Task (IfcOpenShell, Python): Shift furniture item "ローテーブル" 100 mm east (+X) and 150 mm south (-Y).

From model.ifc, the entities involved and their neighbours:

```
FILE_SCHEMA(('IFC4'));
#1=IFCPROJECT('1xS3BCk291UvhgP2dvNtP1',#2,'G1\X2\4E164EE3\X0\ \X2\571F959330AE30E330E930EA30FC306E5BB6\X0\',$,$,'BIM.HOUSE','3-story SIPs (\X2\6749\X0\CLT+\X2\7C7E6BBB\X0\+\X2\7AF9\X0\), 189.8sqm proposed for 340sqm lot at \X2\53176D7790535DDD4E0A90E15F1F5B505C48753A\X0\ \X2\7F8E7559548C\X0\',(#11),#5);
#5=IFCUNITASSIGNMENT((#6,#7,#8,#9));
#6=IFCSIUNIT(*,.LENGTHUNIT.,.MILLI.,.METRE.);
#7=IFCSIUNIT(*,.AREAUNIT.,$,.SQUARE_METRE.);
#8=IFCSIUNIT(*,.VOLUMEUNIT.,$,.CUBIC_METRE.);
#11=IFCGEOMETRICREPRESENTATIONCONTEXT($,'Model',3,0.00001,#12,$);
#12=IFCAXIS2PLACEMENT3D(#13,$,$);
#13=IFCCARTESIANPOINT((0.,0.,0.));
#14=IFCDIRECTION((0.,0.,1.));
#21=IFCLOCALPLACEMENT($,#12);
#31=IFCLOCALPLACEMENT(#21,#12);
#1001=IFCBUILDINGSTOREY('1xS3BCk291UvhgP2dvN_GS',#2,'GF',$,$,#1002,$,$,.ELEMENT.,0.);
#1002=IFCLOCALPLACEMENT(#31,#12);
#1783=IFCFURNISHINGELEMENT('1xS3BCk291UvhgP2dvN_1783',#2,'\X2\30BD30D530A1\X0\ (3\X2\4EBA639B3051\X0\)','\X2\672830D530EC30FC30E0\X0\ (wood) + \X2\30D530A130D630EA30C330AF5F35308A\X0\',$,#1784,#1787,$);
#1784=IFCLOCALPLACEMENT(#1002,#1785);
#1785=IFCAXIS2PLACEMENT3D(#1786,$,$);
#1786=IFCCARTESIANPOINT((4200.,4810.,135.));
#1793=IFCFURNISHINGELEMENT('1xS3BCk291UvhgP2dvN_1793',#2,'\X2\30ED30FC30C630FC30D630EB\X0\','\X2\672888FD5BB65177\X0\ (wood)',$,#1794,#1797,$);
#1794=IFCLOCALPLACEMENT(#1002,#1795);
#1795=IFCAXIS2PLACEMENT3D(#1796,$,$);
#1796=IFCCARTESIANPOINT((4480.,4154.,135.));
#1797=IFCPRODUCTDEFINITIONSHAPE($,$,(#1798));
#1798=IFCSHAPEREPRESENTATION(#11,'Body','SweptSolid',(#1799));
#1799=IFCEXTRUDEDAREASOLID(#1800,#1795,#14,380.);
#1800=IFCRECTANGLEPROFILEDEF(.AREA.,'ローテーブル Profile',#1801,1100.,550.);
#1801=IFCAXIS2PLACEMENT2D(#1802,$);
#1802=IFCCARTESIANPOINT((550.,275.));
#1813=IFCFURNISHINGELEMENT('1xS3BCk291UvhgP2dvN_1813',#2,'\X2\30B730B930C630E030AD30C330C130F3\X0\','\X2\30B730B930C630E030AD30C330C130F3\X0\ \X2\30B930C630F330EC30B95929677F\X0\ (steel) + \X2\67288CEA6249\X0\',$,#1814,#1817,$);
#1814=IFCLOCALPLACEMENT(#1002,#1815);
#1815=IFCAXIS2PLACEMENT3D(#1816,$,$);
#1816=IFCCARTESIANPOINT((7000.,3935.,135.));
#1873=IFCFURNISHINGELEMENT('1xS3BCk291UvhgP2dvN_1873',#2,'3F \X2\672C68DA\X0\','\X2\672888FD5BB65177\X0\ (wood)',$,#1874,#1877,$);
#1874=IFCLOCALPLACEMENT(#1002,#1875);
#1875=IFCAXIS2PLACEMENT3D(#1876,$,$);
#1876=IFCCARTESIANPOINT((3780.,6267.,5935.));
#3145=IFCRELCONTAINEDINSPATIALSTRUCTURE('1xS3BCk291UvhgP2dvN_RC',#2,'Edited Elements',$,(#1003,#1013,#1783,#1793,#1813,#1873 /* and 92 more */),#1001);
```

```python
import ifcopenshell
import ifcopenshell.api.geometry
import ifcopenshell.util.placement
import ifcopenshell.util.unit

model = ifcopenshell.open("model.ifc")
unit_scale = ifcopenshell.util.unit.calculate_unit_scale(model)

item = model.by_guid("1xS3BCk291UvhgP2dvN_1793")
matrix = ifcopenshell.util.placement.get_local_placement(item.ObjectPlacement)
matrix[0, 3] += 0.1 / unit_scale
matrix[1, 3] -= 0.15 / unit_scale
ifcopenshell.api.geometry.edit_object_placement(model, product=item, matrix=matrix, is_si=False)

print(ifcopenshell.util.placement.get_local_placement(item.ObjectPlacement).round(3) + 0.0)

model.write("model-out.ifc")
```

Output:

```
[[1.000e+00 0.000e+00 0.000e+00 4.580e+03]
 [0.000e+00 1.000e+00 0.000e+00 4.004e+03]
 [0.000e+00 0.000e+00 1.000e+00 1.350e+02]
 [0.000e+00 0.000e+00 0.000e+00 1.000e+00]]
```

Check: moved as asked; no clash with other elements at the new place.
